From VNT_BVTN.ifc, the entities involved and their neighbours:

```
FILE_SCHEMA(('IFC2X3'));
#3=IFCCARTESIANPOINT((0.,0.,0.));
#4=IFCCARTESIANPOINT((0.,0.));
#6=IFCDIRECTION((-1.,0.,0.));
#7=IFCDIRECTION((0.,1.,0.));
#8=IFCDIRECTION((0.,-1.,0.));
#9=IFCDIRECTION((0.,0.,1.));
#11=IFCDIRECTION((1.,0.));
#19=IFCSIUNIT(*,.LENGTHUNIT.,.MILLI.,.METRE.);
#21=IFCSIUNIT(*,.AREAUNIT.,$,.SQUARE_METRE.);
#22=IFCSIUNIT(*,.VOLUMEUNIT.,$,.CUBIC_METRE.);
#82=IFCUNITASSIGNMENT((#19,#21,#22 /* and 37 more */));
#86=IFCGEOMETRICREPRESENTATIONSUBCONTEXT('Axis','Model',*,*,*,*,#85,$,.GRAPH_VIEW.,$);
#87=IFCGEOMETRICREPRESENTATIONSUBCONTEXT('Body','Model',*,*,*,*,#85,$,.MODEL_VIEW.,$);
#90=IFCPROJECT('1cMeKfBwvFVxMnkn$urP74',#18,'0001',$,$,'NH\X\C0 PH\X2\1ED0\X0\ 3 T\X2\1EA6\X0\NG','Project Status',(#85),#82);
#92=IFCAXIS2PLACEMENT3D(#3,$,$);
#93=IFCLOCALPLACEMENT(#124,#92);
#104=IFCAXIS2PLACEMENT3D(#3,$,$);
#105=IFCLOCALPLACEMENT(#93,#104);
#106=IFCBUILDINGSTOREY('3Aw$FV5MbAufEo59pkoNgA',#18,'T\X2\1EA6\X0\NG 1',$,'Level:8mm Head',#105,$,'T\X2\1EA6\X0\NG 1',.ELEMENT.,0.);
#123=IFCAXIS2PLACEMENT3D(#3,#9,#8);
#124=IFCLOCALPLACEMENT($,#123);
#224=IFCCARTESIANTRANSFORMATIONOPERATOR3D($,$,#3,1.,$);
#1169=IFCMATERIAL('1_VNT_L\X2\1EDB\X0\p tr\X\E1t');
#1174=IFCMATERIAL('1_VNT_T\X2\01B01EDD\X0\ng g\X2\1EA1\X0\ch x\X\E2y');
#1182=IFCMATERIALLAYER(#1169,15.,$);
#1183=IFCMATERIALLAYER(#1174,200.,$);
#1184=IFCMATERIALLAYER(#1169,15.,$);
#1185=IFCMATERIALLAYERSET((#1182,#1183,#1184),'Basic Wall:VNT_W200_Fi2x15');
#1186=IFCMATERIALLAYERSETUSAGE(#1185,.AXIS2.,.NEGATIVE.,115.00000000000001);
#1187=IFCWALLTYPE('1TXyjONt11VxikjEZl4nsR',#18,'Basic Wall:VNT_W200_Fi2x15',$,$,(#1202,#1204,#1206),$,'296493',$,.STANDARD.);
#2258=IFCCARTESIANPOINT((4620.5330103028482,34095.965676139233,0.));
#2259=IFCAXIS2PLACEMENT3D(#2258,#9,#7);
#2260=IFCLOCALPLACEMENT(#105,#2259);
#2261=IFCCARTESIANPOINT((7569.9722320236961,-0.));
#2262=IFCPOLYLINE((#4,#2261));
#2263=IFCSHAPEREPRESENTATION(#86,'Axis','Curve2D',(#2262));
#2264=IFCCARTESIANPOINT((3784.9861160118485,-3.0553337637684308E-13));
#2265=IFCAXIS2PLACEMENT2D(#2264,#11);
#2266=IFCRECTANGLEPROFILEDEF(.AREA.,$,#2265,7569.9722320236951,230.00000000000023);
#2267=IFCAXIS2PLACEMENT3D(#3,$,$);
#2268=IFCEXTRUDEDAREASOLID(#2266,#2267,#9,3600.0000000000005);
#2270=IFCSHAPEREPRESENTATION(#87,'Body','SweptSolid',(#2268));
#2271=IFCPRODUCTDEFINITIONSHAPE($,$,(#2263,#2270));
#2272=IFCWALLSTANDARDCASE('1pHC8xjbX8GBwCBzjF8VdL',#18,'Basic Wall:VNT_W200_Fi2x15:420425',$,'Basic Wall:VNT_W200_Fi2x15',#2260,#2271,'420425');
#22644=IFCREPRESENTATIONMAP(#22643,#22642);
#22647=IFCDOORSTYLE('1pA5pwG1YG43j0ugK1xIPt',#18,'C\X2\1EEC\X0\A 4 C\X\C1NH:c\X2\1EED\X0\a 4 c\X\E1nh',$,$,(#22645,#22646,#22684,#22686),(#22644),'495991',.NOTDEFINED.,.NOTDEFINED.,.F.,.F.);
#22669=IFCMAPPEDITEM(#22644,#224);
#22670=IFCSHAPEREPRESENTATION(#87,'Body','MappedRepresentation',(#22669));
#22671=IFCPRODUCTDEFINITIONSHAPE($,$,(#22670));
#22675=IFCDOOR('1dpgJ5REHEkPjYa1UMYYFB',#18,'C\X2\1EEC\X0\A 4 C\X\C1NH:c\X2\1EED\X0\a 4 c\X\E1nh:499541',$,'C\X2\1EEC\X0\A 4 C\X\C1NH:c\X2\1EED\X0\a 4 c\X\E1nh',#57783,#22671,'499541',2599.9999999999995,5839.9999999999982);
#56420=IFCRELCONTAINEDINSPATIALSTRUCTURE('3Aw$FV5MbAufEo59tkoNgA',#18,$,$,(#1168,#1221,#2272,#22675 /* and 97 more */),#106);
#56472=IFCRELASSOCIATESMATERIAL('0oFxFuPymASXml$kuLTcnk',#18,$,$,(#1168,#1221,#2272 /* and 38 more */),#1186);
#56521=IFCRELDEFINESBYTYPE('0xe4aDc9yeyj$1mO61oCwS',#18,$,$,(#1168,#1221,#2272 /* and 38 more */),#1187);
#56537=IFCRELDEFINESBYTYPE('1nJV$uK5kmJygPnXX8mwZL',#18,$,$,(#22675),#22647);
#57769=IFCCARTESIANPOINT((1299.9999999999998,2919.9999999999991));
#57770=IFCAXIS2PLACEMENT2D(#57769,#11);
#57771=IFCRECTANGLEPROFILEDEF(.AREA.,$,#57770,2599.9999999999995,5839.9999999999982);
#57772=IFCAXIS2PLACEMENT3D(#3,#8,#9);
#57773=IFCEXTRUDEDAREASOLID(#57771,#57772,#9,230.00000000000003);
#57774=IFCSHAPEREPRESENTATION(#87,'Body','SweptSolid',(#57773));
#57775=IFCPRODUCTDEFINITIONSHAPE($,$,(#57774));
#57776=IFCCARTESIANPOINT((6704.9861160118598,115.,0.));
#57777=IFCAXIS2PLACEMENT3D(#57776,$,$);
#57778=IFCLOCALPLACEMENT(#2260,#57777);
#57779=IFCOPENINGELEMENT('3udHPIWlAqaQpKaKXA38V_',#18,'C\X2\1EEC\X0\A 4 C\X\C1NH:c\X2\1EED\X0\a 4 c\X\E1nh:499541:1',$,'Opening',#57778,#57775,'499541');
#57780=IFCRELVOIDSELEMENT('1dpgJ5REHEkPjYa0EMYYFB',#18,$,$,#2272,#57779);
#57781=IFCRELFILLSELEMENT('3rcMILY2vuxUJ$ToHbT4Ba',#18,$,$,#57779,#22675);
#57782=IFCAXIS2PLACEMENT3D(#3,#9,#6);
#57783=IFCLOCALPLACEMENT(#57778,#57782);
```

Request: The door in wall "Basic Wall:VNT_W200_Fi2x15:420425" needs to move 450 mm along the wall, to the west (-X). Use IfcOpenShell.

```python
import ifcopenshell
import ifcopenshell.api.geometry
import ifcopenshell.util.placement

model = ifcopenshell.open("VNT_BVTN.ifc")

door = model.by_guid("1dpgJ5REHEkPjYa1UMYYFB")
opening = door.FillsVoids[0].RelatingOpeningElement
wall = opening.VoidsElements[0].RelatingBuildingElement

wall_matrix = ifcopenshell.util.placement.get_local_placement(wall.ObjectPlacement)
shift = wall_matrix[:3, 0] * -450.0
before = ifcopenshell.util.placement.get_local_placement(door.ObjectPlacement)[:3, 3].copy()

# The door is placed relative to its opening, so it follows when the opening moves.
matrix = ifcopenshell.util.placement.get_local_placement(opening.ObjectPlacement)
matrix[:3, 3] += shift
ifcopenshell.api.geometry.edit_object_placement(
    model, product=opening, matrix=matrix, is_si=False, should_transform_children=True
)

after = ifcopenshell.util.placement.get_local_placement(door.ObjectPlacement)[:3, 3]
print("door moved by", (after - before).round(3) + 0.0)

model.write("VNT_BVTN-out.ifc")
```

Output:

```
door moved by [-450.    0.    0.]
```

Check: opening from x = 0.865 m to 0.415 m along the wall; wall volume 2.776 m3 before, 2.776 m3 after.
